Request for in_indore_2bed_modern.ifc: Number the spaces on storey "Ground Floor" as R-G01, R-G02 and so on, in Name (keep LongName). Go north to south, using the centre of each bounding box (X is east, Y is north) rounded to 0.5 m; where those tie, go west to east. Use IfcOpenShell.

First a look at what the model holds.

```python
import ifcopenshell
import ifcopenshell.util.element
import ifcopenshell.util.placement

model = ifcopenshell.open("in_indore_2bed_modern.ifc")
print(model.schema)
storey = next(s for s in model.by_type("IfcBuildingStorey") if s.Name == "Ground Floor")
spaces = [e for e in ifcopenshell.util.element.get_decomposition(storey) if e.is_a("IfcSpace")]
for e in sorted(spaces, key=lambda e: e.id()):
    origin = ifcopenshell.util.placement.get_local_placement(e.ObjectPlacement)[:3, 3]
    print(e.id(), e.Name, e.LongName, origin.round(2) + 0.0, sep=" | ")
```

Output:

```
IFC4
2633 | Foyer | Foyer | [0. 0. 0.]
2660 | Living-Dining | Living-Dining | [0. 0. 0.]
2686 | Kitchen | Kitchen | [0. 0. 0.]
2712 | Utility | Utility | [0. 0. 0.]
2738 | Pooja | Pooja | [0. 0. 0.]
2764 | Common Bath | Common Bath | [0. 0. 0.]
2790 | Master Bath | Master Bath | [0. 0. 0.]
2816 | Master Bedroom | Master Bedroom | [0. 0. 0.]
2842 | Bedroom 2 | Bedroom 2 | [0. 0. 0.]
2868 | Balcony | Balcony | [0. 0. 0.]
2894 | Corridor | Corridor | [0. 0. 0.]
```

```python
import ifcopenshell
import ifcopenshell.geom
import ifcopenshell.util.element
import ifcopenshell.util.shape

model = ifcopenshell.open("in_indore_2bed_modern.ifc")
settings = ifcopenshell.geom.settings()
settings.set("use-world-coords", True)


def centre(element):
    shape = ifcopenshell.geom.create_shape(settings, element)
    return ifcopenshell.util.shape.get_bbox_centroid(shape.geometry)


storey = next(s for s in model.by_type("IfcBuildingStorey") if s.Name == "Ground Floor")
spaces = [e for e in ifcopenshell.util.element.get_decomposition(storey) if e.is_a("IfcSpace")]

# Insertion points can sit at a corner or the storey origin, so sort by the geometry (in metres).
centres = {e: centre(e) for e in spaces}
spaces.sort(key=lambda e: (-round(centres[e][1] / 0.5), centres[e][0]))

for i, e in enumerate(spaces, start=1):
    number = f"R-G{i:02d}"
    e.Name = number
    print(e.id(), number)

model.write("in_indore_2bed_modern_updated.ifc")
```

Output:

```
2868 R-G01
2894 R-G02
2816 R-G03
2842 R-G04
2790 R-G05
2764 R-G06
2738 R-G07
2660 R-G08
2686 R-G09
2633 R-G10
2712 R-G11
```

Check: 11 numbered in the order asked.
